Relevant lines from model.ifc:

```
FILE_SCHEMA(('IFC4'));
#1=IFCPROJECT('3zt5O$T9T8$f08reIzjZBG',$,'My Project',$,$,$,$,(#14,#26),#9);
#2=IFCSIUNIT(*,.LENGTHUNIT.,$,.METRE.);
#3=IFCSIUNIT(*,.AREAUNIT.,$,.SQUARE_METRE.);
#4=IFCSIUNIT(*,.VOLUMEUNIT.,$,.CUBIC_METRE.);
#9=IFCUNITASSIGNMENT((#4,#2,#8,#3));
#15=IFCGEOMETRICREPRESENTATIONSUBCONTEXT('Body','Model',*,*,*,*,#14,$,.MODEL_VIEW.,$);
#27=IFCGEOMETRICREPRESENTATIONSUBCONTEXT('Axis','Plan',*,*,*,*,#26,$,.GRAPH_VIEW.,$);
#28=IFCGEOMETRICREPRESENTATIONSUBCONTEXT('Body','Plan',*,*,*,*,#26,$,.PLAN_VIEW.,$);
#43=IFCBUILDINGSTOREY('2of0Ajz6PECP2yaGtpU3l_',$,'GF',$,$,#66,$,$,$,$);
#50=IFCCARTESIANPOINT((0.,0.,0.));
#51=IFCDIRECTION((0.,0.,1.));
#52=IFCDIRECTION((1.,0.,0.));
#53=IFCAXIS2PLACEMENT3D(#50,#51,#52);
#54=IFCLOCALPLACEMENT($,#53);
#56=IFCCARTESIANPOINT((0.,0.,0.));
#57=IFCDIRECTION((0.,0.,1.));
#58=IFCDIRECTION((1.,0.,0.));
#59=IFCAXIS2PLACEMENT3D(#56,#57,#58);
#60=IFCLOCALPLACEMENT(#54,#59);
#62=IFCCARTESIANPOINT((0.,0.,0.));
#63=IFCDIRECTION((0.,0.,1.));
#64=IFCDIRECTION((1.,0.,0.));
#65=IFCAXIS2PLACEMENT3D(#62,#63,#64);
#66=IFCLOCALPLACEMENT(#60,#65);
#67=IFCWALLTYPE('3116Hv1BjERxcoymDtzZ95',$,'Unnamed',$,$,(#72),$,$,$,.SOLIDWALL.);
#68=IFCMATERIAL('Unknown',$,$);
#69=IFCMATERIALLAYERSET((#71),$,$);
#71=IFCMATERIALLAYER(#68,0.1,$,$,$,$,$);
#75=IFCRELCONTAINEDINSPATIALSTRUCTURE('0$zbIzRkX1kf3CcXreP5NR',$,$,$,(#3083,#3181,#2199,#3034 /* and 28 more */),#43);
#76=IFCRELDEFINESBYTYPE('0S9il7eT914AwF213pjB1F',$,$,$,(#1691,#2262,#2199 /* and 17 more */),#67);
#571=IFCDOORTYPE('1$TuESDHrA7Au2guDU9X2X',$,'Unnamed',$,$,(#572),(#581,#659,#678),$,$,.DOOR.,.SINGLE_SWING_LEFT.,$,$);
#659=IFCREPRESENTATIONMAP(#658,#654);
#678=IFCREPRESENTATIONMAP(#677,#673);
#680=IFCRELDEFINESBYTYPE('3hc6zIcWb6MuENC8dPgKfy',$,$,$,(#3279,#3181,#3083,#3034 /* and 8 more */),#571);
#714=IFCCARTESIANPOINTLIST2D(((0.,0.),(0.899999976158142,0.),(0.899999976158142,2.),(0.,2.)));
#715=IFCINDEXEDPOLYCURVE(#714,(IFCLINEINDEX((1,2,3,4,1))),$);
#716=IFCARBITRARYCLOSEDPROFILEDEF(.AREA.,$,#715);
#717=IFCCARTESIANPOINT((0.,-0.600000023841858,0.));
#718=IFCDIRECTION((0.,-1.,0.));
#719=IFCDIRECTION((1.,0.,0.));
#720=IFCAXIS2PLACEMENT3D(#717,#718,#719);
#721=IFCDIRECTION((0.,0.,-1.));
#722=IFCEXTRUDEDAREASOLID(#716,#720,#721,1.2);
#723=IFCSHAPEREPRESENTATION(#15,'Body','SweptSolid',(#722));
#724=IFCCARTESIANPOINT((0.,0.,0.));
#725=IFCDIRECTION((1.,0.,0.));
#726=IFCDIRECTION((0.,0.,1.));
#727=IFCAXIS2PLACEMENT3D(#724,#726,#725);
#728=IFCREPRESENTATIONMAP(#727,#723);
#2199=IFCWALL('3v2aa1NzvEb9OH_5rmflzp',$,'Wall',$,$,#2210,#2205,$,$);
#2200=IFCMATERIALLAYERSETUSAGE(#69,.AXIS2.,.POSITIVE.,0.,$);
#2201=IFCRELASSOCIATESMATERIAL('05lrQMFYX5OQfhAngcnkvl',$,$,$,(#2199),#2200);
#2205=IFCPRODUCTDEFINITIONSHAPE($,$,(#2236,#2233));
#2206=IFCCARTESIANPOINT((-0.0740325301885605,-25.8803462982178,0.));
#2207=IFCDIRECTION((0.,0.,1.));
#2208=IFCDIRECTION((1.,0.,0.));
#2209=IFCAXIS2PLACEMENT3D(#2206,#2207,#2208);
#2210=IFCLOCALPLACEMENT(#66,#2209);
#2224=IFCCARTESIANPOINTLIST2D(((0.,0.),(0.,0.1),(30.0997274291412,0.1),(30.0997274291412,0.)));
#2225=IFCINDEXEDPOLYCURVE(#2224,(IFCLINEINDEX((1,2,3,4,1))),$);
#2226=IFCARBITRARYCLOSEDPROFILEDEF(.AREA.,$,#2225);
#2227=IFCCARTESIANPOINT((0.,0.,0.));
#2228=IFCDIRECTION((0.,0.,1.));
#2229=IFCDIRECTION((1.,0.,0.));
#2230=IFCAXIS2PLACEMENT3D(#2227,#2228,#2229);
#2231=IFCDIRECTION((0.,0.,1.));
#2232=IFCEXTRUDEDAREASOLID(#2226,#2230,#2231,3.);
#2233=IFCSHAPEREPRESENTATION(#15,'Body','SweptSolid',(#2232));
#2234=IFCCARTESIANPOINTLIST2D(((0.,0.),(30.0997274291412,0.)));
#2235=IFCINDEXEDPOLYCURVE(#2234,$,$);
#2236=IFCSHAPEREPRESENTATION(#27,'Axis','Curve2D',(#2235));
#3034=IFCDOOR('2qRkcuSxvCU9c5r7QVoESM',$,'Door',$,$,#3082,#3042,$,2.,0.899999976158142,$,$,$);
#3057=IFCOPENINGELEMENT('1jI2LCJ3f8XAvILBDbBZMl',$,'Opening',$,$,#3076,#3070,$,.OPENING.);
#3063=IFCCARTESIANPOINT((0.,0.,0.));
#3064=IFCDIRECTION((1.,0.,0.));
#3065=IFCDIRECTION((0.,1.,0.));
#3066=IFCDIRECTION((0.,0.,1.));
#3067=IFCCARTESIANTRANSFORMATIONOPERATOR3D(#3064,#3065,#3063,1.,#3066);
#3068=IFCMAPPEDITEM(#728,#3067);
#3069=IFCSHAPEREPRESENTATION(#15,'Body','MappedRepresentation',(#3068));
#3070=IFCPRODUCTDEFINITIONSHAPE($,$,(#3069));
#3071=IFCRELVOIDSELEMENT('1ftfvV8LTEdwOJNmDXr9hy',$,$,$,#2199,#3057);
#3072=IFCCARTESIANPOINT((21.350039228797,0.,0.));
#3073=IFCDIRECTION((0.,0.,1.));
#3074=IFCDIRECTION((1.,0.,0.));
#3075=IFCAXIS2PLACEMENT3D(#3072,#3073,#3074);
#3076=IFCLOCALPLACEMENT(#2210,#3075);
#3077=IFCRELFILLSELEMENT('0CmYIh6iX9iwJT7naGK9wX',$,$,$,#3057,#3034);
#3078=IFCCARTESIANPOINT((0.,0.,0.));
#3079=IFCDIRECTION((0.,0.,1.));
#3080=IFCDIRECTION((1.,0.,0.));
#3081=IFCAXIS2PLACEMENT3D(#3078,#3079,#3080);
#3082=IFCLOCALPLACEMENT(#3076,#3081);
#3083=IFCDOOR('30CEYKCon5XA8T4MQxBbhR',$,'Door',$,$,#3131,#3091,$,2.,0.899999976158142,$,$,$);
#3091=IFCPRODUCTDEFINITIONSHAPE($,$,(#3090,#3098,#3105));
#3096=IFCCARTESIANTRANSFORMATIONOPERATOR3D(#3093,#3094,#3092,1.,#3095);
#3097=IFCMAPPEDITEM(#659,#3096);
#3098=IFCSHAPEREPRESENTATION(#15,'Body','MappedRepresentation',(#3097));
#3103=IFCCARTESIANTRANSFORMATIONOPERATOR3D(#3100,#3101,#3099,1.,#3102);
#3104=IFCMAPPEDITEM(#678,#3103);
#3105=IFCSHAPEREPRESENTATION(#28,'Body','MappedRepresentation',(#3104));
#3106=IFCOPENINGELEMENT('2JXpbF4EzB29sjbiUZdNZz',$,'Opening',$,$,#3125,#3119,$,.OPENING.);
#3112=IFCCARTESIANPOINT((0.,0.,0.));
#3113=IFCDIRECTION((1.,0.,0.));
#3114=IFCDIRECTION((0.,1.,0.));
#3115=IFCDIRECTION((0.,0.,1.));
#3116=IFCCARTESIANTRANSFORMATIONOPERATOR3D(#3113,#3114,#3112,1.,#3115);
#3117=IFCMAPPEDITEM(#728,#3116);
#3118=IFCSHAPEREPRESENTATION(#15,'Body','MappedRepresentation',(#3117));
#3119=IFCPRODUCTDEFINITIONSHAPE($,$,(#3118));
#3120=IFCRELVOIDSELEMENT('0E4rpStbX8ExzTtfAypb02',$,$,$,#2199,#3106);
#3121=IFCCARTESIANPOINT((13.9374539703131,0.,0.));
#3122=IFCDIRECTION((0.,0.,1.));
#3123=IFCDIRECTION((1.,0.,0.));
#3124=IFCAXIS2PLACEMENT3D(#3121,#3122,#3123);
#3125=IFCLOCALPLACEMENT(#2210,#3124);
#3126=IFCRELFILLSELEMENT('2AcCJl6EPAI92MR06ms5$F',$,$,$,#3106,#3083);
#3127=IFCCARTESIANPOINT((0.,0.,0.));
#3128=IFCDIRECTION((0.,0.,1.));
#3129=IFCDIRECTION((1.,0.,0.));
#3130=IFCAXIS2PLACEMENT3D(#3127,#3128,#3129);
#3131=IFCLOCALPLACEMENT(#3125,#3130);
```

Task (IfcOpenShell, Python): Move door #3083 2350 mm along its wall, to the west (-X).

```python
import ifcopenshell
import ifcopenshell.api.geometry
import ifcopenshell.util.placement
import ifcopenshell.util.unit

model = ifcopenshell.open("model.ifc")
unit_scale = ifcopenshell.util.unit.calculate_unit_scale(model)

door = model.by_guid("30CEYKCon5XA8T4MQxBbhR")
opening = door.FillsVoids[0].RelatingOpeningElement
wall = opening.VoidsElements[0].RelatingBuildingElement

wall_matrix = ifcopenshell.util.placement.get_local_placement(wall.ObjectPlacement)
shift = wall_matrix[:3, 0] * -2.35 / unit_scale
before = ifcopenshell.util.placement.get_local_placement(door.ObjectPlacement)[:3, 3].copy()

# The door is placed relative to its opening, so it follows when the opening moves.
matrix = ifcopenshell.util.placement.get_local_placement(opening.ObjectPlacement)
matrix[:3, 3] += shift
ifcopenshell.api.geometry.edit_object_placement(
    model, product=opening, matrix=matrix, is_si=False, should_transform_children=True
)

after = ifcopenshell.util.placement.get_local_placement(door.ObjectPlacement)[:3, 3]
print("door moved by", (after - before).round(3) + 0.0)

model.write("model_edited.ifc")
```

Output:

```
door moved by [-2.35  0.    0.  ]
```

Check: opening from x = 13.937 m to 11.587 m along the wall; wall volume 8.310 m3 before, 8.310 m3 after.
